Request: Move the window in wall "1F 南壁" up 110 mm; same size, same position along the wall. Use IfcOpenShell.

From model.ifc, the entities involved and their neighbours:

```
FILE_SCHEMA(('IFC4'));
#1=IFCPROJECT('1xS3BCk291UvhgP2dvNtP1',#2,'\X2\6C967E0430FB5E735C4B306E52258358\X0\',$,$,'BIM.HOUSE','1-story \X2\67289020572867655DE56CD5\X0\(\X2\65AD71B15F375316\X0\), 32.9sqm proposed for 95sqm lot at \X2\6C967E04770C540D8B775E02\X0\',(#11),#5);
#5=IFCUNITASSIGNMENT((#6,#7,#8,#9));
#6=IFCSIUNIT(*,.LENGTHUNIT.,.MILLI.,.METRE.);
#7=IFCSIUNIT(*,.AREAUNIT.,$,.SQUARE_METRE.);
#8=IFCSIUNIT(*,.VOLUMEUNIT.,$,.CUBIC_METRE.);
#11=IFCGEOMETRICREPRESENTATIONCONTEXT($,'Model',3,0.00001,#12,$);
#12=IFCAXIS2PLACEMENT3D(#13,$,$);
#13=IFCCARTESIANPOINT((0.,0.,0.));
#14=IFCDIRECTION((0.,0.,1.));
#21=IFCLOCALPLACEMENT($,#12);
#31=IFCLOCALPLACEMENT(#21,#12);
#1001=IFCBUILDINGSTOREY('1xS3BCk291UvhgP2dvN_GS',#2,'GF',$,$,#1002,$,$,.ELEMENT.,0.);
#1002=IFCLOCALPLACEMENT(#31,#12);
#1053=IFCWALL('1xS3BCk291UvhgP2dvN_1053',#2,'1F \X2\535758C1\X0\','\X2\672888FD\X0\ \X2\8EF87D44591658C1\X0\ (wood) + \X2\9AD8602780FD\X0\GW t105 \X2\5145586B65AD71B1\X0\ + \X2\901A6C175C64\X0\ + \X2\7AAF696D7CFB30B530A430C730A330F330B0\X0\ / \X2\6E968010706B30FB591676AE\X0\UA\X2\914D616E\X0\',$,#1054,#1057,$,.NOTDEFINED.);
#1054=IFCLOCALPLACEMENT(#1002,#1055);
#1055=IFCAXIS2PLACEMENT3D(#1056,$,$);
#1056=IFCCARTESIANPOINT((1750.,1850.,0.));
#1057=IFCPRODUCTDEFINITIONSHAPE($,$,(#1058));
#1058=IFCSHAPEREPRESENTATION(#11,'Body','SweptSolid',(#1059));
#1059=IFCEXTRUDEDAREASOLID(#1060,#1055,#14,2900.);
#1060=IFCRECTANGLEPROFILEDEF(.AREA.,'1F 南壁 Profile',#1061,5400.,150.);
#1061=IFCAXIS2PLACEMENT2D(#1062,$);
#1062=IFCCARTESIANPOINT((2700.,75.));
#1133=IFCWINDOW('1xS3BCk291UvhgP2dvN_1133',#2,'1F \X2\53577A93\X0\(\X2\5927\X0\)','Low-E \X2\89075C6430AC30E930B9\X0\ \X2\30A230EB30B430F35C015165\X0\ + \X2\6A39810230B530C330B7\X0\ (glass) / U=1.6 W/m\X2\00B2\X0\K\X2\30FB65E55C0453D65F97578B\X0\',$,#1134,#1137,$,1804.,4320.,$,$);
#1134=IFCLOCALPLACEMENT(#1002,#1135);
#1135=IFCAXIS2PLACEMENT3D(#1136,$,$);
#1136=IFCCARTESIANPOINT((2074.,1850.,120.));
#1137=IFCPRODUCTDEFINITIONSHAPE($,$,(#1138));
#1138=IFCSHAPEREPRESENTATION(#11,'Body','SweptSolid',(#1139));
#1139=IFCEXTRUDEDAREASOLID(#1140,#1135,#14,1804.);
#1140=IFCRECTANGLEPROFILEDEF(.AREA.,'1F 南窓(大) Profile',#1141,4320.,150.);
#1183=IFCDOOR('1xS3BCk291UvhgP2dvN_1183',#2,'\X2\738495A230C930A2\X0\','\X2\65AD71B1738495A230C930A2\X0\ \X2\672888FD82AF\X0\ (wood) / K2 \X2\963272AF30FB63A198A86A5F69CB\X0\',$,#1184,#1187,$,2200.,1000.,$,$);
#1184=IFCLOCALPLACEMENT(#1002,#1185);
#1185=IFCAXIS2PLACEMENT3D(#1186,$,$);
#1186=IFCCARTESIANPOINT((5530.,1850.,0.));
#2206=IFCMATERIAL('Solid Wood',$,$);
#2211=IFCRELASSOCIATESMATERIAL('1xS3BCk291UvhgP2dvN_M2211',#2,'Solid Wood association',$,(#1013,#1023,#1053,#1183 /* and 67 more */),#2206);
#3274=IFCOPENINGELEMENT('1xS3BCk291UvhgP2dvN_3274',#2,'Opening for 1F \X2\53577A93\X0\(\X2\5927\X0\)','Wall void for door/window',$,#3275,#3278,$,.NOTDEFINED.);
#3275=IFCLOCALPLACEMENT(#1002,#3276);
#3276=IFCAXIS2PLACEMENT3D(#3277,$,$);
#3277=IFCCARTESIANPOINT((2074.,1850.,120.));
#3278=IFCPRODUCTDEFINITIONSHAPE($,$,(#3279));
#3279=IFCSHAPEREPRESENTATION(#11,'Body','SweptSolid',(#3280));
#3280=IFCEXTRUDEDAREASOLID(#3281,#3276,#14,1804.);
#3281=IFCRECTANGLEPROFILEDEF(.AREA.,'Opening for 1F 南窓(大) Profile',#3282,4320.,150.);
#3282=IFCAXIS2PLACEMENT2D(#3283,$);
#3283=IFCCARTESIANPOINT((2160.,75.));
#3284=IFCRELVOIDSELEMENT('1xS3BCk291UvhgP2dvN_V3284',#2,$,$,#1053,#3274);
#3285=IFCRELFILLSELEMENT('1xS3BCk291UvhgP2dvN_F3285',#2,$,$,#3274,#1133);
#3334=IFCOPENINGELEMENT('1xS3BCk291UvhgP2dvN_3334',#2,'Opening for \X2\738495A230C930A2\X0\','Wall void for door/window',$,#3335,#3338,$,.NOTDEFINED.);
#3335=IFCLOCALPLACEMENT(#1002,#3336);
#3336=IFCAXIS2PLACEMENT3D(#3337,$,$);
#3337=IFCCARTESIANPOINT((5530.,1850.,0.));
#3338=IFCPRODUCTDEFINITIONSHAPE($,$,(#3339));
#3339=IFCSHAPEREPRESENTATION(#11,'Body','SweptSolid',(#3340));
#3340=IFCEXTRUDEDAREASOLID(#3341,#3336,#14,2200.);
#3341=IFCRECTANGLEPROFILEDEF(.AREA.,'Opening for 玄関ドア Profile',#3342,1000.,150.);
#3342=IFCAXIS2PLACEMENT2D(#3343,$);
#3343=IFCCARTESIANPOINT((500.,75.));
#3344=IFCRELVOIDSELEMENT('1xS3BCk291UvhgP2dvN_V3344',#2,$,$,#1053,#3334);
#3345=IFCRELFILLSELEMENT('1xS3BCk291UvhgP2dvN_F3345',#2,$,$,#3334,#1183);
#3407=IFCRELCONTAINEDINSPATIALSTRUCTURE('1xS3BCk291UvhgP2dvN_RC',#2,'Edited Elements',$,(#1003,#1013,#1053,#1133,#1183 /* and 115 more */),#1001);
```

```python
import numpy as np
import ifcopenshell
import ifcopenshell.api.geometry
import ifcopenshell.util.placement
import ifcopenshell.util.unit

model = ifcopenshell.open("model.ifc")
unit_scale = ifcopenshell.util.unit.calculate_unit_scale(model)

window = model.by_guid("1xS3BCk291UvhgP2dvN_1133")
opening = window.FillsVoids[0].RelatingOpeningElement
dz = 0.11 / unit_scale

shift = np.array([0.0, 0.0, dz])
# The window is not placed relative to its opening, so move both.
for product in (opening, window):
    matrix = ifcopenshell.util.placement.get_local_placement(product.ObjectPlacement)
    matrix[:3, 3] += shift
    ifcopenshell.api.geometry.edit_object_placement(model, product=product, matrix=matrix, is_si=False)

print(f"moved by {dz * unit_scale:+.3f} m")

model.write("model-out.ifc")
```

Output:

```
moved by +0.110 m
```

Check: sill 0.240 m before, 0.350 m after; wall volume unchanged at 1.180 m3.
